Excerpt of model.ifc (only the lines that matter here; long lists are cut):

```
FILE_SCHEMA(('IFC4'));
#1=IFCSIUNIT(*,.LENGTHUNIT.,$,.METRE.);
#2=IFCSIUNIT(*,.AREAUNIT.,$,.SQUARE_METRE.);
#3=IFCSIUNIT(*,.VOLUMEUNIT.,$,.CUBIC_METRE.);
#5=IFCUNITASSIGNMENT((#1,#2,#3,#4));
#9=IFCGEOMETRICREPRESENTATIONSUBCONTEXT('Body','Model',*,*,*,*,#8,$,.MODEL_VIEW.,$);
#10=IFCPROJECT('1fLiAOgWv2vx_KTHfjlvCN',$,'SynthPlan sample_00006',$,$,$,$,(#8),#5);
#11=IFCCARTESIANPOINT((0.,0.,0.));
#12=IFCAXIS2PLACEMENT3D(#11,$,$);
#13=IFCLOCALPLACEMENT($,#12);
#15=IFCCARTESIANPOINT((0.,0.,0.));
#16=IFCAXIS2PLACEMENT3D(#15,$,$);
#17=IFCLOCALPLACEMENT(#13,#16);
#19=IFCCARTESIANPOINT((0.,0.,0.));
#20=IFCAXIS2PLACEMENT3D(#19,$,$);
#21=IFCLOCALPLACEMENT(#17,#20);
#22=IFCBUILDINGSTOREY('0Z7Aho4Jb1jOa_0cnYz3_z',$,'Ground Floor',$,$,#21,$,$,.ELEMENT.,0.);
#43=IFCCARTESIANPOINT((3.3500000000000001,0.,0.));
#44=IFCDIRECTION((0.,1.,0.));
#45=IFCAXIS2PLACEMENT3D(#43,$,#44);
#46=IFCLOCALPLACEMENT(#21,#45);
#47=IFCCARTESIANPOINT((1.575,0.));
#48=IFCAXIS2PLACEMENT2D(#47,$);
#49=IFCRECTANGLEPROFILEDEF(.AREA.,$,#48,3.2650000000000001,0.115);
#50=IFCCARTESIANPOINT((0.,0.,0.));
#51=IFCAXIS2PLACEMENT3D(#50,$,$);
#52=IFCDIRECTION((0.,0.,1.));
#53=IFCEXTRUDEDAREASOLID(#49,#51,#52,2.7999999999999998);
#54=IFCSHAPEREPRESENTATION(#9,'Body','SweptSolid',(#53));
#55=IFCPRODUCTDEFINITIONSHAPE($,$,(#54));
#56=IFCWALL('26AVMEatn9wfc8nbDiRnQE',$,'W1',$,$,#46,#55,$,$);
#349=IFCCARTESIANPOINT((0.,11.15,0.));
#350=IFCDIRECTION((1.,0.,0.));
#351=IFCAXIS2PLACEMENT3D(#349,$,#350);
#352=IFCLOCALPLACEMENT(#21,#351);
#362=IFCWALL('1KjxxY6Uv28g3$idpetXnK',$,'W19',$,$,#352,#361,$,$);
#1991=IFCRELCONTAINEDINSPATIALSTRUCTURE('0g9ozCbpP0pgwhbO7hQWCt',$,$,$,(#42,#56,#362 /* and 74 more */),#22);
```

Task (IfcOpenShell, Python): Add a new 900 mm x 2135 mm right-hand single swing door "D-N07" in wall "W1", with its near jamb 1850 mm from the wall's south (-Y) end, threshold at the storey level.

```python
import numpy as np
import ifcopenshell
import ifcopenshell.api.feature
import ifcopenshell.api.geometry
import ifcopenshell.api.root
import ifcopenshell.api.spatial
import ifcopenshell.geom
import ifcopenshell.util.element
import ifcopenshell.util.placement
import ifcopenshell.util.representation
import ifcopenshell.util.shape
import ifcopenshell.util.unit

model = ifcopenshell.open("model.ifc")
unit_scale = ifcopenshell.util.unit.calculate_unit_scale(model)
settings = ifcopenshell.geom.settings()


def volume(element):
    """Net volume in cubic metres, openings subtracted."""
    shape = ifcopenshell.geom.create_shape(settings, element)
    return ifcopenshell.util.shape.get_volume(shape.geometry)


wall = model.by_guid("26AVMEatn9wfc8nbDiRnQE")
storey = ifcopenshell.util.element.get_container(wall, ifc_class="IfcBuildingStorey")
context = ifcopenshell.util.representation.get_context(model, "Model", "Body", "MODEL_VIEW")
before = volume(wall)

width, height, from_end, sill = 0.9, 2.135, 1.85, 0.0  # metres

# The wall runs along its own X axis, and the end named is its -X end.
wall_shape = ifcopenshell.geom.create_shape(settings, wall)
x, y, z = ifcopenshell.util.shape.get_vertices(wall_shape.geometry).T
start = x.min() + from_end
face, thickness = float(y.min()), float(y.max() - y.min())
wall_matrix = ifcopenshell.util.placement.get_local_placement(wall.ObjectPlacement)
level = ifcopenshell.util.placement.get_local_placement(storey.ObjectPlacement)[2, 3]


def in_wall(x, y):
    """Placement at x, y metres in the wall's axes, at sill height."""
    matrix = wall_matrix.copy()
    matrix[:, 3] = wall_matrix @ np.array([x / unit_scale, y / unit_scale, 0.0, 1.0])
    matrix[2, 3] = level + sill / unit_scale
    return matrix


# Opening: a box that overshoots both wall faces by 50 mm.
opening = ifcopenshell.api.root.create_entity(model, ifc_class="IfcOpeningElement", predefined_type="OPENING")
box = ifcopenshell.api.geometry.add_wall_representation(
    model, context=context, length=width, height=height, thickness=thickness + 0.1
)
ifcopenshell.api.geometry.assign_representation(model, product=opening, representation=box)
ifcopenshell.api.geometry.edit_object_placement(model, product=opening, matrix=in_wall(start, face - 0.05), is_si=False)
ifcopenshell.api.feature.add_feature(model, feature=opening, element=wall)

door = ifcopenshell.api.root.create_entity(model, ifc_class="IfcDoor", name="D-N07", predefined_type="DOOR")
door.OverallWidth, door.OverallHeight = width / unit_scale, height / unit_scale
door.OperationType = "SINGLE_SWING_RIGHT"
body = ifcopenshell.api.geometry.add_door_representation(
    model,
    context=context,
    overall_width=door.OverallWidth,
    overall_height=door.OverallHeight,
    operation_type="SINGLE_SWING_RIGHT",
    lining_properties={"LiningDepth": thickness / unit_scale, "ThresholdDepth": thickness / unit_scale},
)
ifcopenshell.api.geometry.assign_representation(model, product=door, representation=body)
ifcopenshell.api.spatial.assign_container(model, products=[door], relating_structure=storey)
ifcopenshell.api.feature.add_filling(model, opening=opening, element=door)

# The lining spans the wall, so the door starts at the wall face.
ifcopenshell.api.geometry.edit_object_placement(model, product=door, matrix=in_wall(start, face), is_si=False)

after = volume(wall)

print(f"wall volume {before:.3f} -> {after:.3f} m3")

model.write("model_updated.ifc")
```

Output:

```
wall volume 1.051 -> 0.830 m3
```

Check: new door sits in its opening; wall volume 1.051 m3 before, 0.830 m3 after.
